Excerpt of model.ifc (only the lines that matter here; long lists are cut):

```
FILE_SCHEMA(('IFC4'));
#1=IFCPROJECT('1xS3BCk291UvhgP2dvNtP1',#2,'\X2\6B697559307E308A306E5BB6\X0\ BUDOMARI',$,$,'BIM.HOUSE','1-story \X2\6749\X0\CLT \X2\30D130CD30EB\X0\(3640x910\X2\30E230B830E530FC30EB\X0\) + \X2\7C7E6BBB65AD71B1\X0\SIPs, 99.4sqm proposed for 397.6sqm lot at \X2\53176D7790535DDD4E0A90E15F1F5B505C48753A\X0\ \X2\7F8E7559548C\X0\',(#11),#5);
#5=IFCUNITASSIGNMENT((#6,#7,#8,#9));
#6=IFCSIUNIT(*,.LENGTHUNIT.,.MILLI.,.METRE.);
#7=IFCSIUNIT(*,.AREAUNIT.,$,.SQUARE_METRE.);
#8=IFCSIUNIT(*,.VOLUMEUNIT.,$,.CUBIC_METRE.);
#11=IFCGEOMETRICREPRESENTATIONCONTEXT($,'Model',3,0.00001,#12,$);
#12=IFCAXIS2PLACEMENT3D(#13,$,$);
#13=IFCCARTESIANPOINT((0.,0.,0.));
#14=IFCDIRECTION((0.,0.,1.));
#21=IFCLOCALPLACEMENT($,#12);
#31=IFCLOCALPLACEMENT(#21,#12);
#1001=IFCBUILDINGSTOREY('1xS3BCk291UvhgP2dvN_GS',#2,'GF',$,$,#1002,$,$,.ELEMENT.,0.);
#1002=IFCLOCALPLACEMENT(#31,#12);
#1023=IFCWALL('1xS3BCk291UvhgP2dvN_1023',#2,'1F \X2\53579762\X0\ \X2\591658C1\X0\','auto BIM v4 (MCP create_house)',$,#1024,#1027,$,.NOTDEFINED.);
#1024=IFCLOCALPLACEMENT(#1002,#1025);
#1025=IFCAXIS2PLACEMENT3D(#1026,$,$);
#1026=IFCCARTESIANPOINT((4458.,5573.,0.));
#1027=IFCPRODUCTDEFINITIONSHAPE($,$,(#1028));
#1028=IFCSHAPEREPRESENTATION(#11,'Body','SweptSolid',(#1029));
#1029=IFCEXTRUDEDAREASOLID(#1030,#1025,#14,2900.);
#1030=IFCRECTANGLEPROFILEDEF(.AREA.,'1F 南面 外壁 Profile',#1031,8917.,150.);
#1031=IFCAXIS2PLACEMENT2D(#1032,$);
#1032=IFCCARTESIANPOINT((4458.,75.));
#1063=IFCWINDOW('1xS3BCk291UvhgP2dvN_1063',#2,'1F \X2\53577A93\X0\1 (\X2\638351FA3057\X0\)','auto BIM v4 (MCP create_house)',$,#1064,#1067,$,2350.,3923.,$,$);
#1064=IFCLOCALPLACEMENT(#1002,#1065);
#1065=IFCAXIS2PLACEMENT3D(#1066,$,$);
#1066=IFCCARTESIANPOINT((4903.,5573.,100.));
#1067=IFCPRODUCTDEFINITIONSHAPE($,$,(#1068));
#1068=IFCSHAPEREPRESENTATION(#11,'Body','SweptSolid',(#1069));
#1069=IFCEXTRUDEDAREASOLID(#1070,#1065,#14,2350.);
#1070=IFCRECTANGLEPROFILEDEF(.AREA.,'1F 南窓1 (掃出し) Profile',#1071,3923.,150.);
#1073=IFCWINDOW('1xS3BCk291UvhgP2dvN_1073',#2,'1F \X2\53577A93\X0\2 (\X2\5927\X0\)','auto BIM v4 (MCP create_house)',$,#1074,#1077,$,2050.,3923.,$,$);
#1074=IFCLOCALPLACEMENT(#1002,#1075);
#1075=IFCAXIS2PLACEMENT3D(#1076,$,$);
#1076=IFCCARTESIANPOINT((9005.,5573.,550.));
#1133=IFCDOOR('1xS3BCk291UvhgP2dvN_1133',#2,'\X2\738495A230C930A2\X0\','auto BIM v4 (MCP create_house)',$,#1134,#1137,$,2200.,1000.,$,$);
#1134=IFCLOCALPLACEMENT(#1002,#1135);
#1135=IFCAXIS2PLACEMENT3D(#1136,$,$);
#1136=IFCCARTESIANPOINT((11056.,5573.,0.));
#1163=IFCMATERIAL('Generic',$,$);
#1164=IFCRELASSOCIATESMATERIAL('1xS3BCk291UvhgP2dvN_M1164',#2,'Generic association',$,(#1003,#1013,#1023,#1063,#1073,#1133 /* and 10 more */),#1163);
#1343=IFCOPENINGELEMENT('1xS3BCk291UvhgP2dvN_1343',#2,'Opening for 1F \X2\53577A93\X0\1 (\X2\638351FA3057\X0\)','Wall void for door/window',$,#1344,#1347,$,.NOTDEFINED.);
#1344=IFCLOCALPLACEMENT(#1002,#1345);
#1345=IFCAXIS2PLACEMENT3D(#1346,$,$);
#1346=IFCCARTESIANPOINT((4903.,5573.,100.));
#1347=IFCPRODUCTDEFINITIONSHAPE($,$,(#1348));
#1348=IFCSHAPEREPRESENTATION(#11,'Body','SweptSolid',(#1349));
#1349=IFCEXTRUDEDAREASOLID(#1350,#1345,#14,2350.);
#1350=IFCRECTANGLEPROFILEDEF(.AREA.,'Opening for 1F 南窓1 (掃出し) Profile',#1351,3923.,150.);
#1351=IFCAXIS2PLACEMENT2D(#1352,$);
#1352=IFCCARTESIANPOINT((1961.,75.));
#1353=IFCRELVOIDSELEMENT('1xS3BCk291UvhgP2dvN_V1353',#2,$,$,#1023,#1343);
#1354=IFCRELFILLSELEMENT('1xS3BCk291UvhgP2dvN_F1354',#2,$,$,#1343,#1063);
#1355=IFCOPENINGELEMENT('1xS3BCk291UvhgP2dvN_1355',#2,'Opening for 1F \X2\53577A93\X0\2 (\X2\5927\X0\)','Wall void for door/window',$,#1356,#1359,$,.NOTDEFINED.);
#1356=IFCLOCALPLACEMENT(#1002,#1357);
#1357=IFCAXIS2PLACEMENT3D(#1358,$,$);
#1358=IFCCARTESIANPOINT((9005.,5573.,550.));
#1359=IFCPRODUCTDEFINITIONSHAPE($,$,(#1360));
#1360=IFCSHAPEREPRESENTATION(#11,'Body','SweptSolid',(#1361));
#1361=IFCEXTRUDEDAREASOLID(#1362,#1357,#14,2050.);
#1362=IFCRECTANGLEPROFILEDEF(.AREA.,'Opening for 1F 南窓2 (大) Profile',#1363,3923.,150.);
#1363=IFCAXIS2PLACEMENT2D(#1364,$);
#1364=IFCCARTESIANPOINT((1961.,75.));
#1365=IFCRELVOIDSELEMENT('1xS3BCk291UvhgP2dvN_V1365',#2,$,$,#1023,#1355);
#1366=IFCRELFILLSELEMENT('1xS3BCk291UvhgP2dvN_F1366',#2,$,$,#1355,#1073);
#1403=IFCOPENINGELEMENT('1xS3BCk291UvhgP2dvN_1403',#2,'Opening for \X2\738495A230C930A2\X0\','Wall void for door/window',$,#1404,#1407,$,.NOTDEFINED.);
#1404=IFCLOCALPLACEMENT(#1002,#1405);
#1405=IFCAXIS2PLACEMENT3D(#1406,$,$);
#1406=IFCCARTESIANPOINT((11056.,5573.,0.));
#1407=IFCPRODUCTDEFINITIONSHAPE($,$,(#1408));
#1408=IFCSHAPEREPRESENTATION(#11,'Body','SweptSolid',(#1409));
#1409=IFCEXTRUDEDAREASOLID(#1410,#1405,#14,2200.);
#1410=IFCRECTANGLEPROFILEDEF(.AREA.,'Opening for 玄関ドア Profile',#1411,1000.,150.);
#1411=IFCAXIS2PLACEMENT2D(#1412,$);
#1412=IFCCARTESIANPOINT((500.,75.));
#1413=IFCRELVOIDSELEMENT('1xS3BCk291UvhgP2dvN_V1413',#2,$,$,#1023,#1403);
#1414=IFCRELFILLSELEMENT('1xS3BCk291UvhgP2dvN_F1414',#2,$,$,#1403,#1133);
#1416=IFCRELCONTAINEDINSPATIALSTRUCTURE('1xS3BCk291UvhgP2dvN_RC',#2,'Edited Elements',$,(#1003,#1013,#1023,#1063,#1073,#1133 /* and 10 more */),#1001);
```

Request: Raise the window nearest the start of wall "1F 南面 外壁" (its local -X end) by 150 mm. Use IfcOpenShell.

```python
import numpy as np
import ifcopenshell
import ifcopenshell.api.geometry
import ifcopenshell.util.placement
import ifcopenshell.util.unit

model = ifcopenshell.open("model.ifc")
unit_scale = ifcopenshell.util.unit.calculate_unit_scale(model)

window = model.by_id(1063)
opening = window.FillsVoids[0].RelatingOpeningElement
dz = 0.15 / unit_scale

shift = np.array([0.0, 0.0, dz])
# The window is not placed relative to its opening, so move both.
for product in (opening, window):
    matrix = ifcopenshell.util.placement.get_local_placement(product.ObjectPlacement)
    matrix[:3, 3] += shift
    ifcopenshell.api.geometry.edit_object_placement(model, product=product, matrix=matrix, is_si=False)

print(f"moved by {dz * unit_scale:+.3f} m")

model.write("model_rev.ifc")
```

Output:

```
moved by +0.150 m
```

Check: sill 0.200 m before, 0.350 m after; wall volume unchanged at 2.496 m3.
